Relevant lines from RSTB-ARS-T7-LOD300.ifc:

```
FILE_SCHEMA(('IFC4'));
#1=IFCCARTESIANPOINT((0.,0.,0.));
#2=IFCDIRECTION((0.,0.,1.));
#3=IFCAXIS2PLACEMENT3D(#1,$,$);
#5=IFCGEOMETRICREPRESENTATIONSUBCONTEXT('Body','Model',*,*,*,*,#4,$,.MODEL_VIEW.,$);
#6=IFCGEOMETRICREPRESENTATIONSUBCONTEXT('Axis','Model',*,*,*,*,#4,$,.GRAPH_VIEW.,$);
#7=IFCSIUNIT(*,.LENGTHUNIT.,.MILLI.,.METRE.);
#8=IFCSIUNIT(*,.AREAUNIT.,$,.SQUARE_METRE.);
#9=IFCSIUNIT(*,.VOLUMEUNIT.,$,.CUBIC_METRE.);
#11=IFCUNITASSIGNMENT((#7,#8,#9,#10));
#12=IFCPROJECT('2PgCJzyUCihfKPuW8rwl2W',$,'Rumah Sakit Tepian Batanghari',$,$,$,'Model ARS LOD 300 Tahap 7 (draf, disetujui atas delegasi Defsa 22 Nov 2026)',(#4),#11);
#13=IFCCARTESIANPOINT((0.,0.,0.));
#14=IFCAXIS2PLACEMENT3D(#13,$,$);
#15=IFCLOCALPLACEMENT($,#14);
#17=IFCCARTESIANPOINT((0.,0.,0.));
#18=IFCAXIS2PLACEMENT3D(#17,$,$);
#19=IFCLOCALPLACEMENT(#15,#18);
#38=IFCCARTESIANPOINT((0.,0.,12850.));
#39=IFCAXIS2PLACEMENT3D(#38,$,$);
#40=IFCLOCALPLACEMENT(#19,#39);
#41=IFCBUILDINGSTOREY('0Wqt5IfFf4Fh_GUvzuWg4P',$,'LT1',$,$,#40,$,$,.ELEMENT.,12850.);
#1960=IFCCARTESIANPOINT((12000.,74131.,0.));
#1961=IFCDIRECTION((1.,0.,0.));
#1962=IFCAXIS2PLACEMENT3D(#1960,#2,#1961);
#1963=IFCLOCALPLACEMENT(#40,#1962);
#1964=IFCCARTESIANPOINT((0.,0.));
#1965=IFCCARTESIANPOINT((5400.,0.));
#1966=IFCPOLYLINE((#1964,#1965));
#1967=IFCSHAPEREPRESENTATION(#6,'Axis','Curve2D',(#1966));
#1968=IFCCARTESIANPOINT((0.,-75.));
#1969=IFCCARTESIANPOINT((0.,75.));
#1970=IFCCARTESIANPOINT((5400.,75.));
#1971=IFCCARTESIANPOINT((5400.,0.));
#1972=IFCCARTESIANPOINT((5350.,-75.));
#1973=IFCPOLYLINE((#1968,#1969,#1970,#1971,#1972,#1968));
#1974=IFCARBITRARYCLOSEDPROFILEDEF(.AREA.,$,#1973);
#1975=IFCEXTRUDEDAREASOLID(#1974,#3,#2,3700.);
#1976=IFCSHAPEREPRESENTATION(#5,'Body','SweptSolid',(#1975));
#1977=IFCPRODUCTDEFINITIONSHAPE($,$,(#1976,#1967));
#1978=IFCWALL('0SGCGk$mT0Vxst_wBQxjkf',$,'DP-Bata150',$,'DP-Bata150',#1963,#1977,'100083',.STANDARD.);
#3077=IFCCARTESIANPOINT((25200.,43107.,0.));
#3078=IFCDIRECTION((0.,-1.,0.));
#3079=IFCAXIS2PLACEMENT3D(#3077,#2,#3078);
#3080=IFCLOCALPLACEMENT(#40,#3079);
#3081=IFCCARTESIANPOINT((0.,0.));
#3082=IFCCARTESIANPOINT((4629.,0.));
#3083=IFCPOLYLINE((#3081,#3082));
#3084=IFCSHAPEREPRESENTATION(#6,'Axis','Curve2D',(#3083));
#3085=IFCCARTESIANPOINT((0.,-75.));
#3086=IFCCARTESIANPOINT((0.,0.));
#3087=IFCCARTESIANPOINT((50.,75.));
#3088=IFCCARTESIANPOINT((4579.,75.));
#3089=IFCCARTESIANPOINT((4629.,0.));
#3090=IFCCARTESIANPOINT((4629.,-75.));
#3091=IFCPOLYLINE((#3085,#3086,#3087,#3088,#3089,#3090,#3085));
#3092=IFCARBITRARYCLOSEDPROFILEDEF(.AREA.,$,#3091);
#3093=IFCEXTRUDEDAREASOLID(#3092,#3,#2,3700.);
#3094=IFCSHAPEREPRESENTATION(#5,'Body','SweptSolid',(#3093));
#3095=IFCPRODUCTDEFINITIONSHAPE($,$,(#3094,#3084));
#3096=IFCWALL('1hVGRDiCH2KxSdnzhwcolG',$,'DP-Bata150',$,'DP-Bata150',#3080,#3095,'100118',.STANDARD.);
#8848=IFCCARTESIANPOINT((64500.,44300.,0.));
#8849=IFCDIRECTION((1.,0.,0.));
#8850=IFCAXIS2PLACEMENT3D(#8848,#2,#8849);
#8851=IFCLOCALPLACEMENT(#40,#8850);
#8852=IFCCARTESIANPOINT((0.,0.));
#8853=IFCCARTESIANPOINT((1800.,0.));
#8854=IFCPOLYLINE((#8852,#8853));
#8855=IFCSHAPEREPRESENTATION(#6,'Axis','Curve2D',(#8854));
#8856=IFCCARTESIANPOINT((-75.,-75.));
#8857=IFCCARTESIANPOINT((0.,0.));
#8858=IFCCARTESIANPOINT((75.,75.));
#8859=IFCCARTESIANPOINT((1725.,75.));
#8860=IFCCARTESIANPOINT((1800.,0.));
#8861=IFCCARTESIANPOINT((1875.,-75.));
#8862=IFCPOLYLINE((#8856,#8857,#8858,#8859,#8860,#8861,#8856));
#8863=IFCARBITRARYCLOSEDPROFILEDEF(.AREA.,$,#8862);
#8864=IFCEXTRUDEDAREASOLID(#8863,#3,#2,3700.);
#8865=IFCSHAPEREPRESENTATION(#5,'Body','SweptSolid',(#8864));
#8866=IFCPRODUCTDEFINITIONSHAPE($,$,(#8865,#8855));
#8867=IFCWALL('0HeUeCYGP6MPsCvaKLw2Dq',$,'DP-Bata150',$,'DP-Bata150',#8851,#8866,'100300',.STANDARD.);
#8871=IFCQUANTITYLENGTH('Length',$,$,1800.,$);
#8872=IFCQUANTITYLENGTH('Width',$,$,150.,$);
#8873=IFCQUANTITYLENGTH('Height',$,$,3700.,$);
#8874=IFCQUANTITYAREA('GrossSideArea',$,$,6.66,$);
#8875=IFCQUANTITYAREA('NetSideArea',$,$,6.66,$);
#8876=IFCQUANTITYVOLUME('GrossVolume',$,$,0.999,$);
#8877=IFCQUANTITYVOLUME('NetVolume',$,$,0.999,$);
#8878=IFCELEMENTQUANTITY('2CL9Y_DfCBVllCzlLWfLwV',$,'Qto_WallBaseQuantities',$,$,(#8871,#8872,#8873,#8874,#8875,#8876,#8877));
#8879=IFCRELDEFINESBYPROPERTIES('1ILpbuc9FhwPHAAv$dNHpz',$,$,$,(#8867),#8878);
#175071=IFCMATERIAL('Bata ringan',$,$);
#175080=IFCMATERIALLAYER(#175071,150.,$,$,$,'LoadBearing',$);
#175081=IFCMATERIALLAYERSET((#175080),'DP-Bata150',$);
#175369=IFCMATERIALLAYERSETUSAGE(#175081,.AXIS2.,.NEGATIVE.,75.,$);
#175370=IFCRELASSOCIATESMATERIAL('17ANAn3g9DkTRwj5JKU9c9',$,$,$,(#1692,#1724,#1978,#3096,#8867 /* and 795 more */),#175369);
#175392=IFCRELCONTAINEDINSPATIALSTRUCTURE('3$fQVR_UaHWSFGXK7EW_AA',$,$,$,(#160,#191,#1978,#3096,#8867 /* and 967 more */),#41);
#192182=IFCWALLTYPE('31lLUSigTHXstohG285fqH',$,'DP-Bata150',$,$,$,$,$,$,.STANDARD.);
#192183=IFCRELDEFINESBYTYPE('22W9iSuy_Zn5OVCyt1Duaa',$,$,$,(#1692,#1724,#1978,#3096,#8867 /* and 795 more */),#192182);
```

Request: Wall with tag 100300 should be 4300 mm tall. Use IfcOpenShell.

```python
import ifcopenshell
import ifcopenshell.api.pset
import ifcopenshell.geom
import ifcopenshell.util.element
import ifcopenshell.util.representation
import ifcopenshell.util.shape
import ifcopenshell.util.unit

model = ifcopenshell.open("RSTB-ARS-T7-LOD300.ifc")
unit_scale = ifcopenshell.util.unit.calculate_unit_scale(model)
area_scale = ifcopenshell.util.unit.calculate_unit_scale(model, "AREAUNIT")
volume_scale = ifcopenshell.util.unit.calculate_unit_scale(model, "VOLUMEUNIT")
settings = ifcopenshell.geom.settings()


def volume(element):
    """Net volume in cubic metres, openings subtracted."""
    shape = ifcopenshell.geom.create_shape(settings, element)
    return ifcopenshell.util.shape.get_volume(shape.geometry)


wall = model.by_id(8867)
before = volume(wall)

body = ifcopenshell.util.representation.get_representation(wall, "Model", "Body")
solid = body.Items[0]
old_height = solid.Depth
solid.Depth = 4.3 / unit_scale
after = volume(wall)
thickness = 0.15  # wall thickness in metres

# Update the stored height, areas and volumes.
qto = model.by_id(ifcopenshell.util.element.get_pset(wall, "Qto_WallBaseQuantities", should_inherit=False)["id"])
ifcopenshell.api.pset.edit_qto(model, qto=qto, properties={
    "Height": solid.Depth,
    "GrossSideArea": ifcopenshell.util.element.get_pset(wall, "Qto_WallBaseQuantities", "GrossSideArea") * solid.Depth / old_height,
    "NetSideArea": after / thickness / area_scale,
    "GrossVolume": ifcopenshell.util.element.get_pset(wall, "Qto_WallBaseQuantities", "GrossVolume") * solid.Depth / old_height,
    "NetVolume": after / volume_scale,
})

print(f"height {old_height:g} -> {solid.Depth:g}, volume {before:.3f} -> {after:.3f} m3")

model.write("RSTB-ARS-T7-LOD300_updated.ifc")
```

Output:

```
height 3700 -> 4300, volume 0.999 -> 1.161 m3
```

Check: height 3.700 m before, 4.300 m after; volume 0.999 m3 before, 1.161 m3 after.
